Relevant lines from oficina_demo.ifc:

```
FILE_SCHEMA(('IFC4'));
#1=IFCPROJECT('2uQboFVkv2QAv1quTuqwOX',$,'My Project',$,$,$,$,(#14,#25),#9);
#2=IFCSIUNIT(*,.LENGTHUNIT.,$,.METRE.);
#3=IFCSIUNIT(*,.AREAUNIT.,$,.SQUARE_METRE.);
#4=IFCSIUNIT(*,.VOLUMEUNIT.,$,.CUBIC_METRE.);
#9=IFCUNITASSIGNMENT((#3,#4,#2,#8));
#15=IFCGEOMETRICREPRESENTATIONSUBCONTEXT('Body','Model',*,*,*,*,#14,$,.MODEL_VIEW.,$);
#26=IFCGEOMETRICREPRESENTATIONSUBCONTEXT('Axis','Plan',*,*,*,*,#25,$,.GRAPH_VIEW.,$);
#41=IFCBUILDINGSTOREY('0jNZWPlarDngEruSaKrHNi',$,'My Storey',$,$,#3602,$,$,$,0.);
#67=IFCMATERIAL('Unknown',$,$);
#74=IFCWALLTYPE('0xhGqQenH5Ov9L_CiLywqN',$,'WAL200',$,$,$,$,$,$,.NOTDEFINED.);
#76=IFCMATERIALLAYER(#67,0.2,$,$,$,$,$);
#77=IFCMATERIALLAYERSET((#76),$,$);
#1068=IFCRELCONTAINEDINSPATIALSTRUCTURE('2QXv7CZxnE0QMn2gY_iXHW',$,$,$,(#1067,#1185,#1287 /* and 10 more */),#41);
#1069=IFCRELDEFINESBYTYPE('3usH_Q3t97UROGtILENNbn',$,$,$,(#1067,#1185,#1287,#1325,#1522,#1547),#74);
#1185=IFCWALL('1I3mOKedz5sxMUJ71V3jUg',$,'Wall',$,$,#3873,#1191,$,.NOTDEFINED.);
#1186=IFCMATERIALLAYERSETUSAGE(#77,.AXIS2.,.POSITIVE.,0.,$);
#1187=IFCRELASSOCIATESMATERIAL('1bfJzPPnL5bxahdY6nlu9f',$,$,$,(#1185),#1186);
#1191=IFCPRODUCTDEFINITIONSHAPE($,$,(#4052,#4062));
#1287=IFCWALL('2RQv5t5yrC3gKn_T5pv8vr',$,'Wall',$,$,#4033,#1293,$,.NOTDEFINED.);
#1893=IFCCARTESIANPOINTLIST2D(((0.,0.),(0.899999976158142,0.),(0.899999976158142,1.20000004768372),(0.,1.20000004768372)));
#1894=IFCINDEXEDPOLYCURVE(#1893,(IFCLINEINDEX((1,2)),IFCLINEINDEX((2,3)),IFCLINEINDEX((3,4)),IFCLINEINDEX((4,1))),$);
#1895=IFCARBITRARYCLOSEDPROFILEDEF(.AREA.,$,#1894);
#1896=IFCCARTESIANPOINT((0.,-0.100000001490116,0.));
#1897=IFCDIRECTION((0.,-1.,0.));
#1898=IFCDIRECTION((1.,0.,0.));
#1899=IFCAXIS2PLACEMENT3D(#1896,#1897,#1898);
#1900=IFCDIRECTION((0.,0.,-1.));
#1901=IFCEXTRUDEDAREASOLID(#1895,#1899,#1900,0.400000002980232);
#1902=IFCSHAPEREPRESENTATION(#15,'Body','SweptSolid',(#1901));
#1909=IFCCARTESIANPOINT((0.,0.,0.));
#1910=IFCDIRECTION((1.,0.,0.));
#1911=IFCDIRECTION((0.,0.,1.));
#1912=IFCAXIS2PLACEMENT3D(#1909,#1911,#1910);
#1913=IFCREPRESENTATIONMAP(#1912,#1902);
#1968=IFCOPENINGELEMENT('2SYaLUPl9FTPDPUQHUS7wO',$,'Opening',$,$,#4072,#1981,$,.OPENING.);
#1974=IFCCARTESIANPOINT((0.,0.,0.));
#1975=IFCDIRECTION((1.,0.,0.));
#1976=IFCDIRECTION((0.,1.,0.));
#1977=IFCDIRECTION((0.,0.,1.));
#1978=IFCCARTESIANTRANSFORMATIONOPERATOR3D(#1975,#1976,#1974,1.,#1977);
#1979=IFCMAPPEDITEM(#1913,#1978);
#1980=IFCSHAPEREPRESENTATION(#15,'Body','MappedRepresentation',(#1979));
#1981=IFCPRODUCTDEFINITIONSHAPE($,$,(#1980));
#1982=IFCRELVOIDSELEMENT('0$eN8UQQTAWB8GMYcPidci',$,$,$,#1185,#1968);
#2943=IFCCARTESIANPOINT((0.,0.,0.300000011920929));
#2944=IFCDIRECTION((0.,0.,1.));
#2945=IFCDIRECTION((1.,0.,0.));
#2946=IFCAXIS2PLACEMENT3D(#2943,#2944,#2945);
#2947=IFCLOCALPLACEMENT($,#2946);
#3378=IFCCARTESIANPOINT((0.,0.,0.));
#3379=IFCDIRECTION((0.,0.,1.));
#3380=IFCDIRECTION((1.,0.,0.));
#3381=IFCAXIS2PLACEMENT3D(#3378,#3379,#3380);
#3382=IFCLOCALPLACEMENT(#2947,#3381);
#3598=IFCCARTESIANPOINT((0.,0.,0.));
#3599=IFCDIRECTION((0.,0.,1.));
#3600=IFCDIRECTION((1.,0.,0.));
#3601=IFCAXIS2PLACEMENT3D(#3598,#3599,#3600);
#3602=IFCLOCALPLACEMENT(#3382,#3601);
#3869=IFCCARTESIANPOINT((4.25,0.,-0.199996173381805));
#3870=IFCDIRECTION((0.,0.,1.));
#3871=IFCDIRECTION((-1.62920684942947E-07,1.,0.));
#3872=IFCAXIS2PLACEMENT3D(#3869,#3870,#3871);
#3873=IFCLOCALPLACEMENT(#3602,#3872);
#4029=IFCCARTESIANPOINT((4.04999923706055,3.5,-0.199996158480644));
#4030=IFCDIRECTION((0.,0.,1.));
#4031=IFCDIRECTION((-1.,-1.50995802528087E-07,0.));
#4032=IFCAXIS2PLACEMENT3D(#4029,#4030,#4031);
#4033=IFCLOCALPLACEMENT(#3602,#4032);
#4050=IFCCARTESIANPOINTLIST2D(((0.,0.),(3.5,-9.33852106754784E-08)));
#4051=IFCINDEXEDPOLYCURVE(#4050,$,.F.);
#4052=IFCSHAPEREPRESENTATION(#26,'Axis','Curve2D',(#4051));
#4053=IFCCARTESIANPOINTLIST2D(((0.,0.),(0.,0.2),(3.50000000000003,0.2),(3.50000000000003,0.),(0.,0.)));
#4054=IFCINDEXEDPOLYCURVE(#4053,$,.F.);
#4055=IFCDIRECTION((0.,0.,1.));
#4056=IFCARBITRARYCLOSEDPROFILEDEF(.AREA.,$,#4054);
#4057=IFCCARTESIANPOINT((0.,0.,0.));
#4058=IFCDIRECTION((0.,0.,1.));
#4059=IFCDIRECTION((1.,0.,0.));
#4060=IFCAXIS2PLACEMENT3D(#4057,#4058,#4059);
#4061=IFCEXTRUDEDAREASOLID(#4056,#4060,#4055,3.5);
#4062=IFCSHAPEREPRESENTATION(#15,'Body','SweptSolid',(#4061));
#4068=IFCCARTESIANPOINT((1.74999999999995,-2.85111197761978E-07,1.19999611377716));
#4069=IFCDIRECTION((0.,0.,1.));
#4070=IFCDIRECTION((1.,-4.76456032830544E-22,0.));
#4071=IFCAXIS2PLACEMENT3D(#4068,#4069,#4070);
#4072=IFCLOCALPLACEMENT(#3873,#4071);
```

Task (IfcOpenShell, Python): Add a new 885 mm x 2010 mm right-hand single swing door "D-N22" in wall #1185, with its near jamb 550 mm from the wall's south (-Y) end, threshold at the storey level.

```python
import numpy as np
import ifcopenshell
import ifcopenshell.api.feature
import ifcopenshell.api.geometry
import ifcopenshell.api.root
import ifcopenshell.api.spatial
import ifcopenshell.geom
import ifcopenshell.util.element
import ifcopenshell.util.placement
import ifcopenshell.util.representation
import ifcopenshell.util.shape
import ifcopenshell.util.unit

model = ifcopenshell.open("oficina_demo.ifc")
unit_scale = ifcopenshell.util.unit.calculate_unit_scale(model)
settings = ifcopenshell.geom.settings()


def volume(element):
    """Net volume in cubic metres, openings subtracted."""
    shape = ifcopenshell.geom.create_shape(settings, element)
    return ifcopenshell.util.shape.get_volume(shape.geometry)


wall = model.by_id(1185)
storey = ifcopenshell.util.element.get_container(wall, ifc_class="IfcBuildingStorey")
context = ifcopenshell.util.representation.get_context(model, "Model", "Body", "MODEL_VIEW")
before = volume(wall)

width, height, from_end, sill = 0.885, 2.01, 0.55, 0.0  # metres

# The wall runs along its own X axis, and the end named is its -X end.
wall_shape = ifcopenshell.geom.create_shape(settings, wall)
x, y, z = ifcopenshell.util.shape.get_vertices(wall_shape.geometry).T
start = x.min() + from_end
face, thickness = float(y.min()), float(y.max() - y.min())
wall_matrix = ifcopenshell.util.placement.get_local_placement(wall.ObjectPlacement)
level = ifcopenshell.util.placement.get_local_placement(storey.ObjectPlacement)[2, 3]


def in_wall(x, y):
    """Placement at x, y metres in the wall's axes, at sill height."""
    matrix = wall_matrix.copy()
    matrix[:, 3] = wall_matrix @ np.array([x / unit_scale, y / unit_scale, 0.0, 1.0])
    matrix[2, 3] = level + sill / unit_scale
    return matrix


# Opening: a box that overshoots both wall faces by 50 mm.
opening = ifcopenshell.api.root.create_entity(model, ifc_class="IfcOpeningElement", predefined_type="OPENING")
box = ifcopenshell.api.geometry.add_wall_representation(
    model, context=context, length=width, height=height, thickness=thickness + 0.1
)
ifcopenshell.api.geometry.assign_representation(model, product=opening, representation=box)
ifcopenshell.api.geometry.edit_object_placement(model, product=opening, matrix=in_wall(start, face - 0.05), is_si=False)
ifcopenshell.api.feature.add_feature(model, feature=opening, element=wall)

door = ifcopenshell.api.root.create_entity(model, ifc_class="IfcDoor", name="D-N22", predefined_type="DOOR")
door.OverallWidth, door.OverallHeight = width / unit_scale, height / unit_scale
door.OperationType = "SINGLE_SWING_RIGHT"
body = ifcopenshell.api.geometry.add_door_representation(
    model,
    context=context,
    overall_width=door.OverallWidth,
    overall_height=door.OverallHeight,
    operation_type="SINGLE_SWING_RIGHT",
    lining_properties={"LiningDepth": thickness / unit_scale, "ThresholdDepth": thickness / unit_scale},
)
ifcopenshell.api.geometry.assign_representation(model, product=door, representation=body)
ifcopenshell.api.spatial.assign_container(model, products=[door], relating_structure=storey)
ifcopenshell.api.feature.add_filling(model, opening=opening, element=door)

# The lining spans the wall, so the door starts at the wall face.
ifcopenshell.api.geometry.edit_object_placement(model, product=door, matrix=in_wall(start, face), is_si=False)

after = volume(wall)

print(f"wall volume {before:.3f} -> {after:.3f} m3")

model.write("oficina_demo_rev.ifc")
```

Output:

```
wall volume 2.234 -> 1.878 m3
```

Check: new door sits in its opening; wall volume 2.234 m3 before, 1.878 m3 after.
